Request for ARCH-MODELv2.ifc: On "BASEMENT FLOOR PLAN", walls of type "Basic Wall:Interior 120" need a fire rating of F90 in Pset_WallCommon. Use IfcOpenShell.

First a look at what the model holds.

```python
import ifcopenshell
import ifcopenshell.util.element

model = ifcopenshell.open("ARCH-MODELv2.ifc")
print(model.schema)
storey = next(s for s in model.by_type("IfcBuildingStorey") if s.Name == "BASEMENT FLOOR PLAN")
walls = [e for e in ifcopenshell.util.element.get_decomposition(storey) if e.is_a("IfcWall")]
seen = {}
for e in walls:
    element_type = ifcopenshell.util.element.get_type(e)
    key = (element_type.Name if element_type != e and element_type else None, ifcopenshell.util.element.get_pset(e, "Pset_WallCommon", "FireRating"))
    seen[key] = seen.get(key, 0) + 1
for (name, value), count in sorted(seen.items(), key=str):
    print(count, "x", name, "|", value)
```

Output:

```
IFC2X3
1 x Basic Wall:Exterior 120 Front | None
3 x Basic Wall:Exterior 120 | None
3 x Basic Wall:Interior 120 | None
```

```python
import ifcopenshell
import ifcopenshell.api.pset
import ifcopenshell.util.element

model = ifcopenshell.open("ARCH-MODELv2.ifc")

storey = next(s for s in model.by_type("IfcBuildingStorey") if s.Name == "BASEMENT FLOOR PLAN")
walls = [e for e in ifcopenshell.util.element.get_decomposition(storey) if e.is_a("IfcWall")]

count = 0
for e in walls:
    element_type = ifcopenshell.util.element.get_type(e)
    if element_type in (None, e) or element_type.Name != "Basic Wall:Interior 120":
        continue
    # add_pset returns the element's existing set when there is one.
    pset = ifcopenshell.api.pset.add_pset(model, product=e, name="Pset_WallCommon")
    ifcopenshell.api.pset.edit_pset(model, pset=pset, properties={"FireRating": "F90"})
    count += 1

print(count, "walls updated")

model.write("ARCH-MODELv2_rev.ifc")
```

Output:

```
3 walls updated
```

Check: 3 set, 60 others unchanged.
